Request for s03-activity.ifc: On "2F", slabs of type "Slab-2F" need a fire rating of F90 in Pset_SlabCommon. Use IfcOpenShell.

First a look at what the model holds.

```python
import ifcopenshell
import ifcopenshell.util.element

model = ifcopenshell.open("s03-activity.ifc")
print(model.schema)
storey = next(s for s in model.by_type("IfcBuildingStorey") if s.Name == "2F")
slabs = [e for e in ifcopenshell.util.element.get_decomposition(storey) if e.is_a("IfcSlab")]
seen = {}
for e in slabs:
    element_type = ifcopenshell.util.element.get_type(e)
    key = (element_type.Name if element_type != e and element_type else None, ifcopenshell.util.element.get_pset(e, "Pset_SlabCommon", "FireRating"))
    seen[key] = seen.get(key, 0) + 1
for (name, value), count in sorted(seen.items(), key=str):
    print(count, "x", name, "|", value)
```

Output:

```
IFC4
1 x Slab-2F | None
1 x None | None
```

```python
import ifcopenshell
import ifcopenshell.api.pset
import ifcopenshell.util.element

model = ifcopenshell.open("s03-activity.ifc")

storey = next(s for s in model.by_type("IfcBuildingStorey") if s.Name == "2F")
slabs = [e for e in ifcopenshell.util.element.get_decomposition(storey) if e.is_a("IfcSlab")]

count = 0
for e in slabs:
    element_type = ifcopenshell.util.element.get_type(e)
    if element_type in (None, e) or element_type.Name != "Slab-2F":
        continue
    # add_pset returns the element's existing set when there is one.
    pset = ifcopenshell.api.pset.add_pset(model, product=e, name="Pset_SlabCommon")
    ifcopenshell.api.pset.edit_pset(model, pset=pset, properties={"FireRating": "F90"})
    count += 1

print(count, "slabs updated")

model.write("s03-activity_rev.ifc")
```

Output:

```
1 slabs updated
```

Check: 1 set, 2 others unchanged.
